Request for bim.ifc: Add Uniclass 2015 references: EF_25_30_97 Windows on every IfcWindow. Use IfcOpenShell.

First a look at what the model holds.

```python
import ifcopenshell

model = ifcopenshell.open("bim.ifc")
print(model.schema)
print("classifications:", [c.Name for c in model.by_type("IfcClassification")])
for ifc_class in ("IfcDoor", "IfcRoof", "IfcStair", "IfcWall", "IfcWindow"):
    print(ifc_class, len(model.by_type(ifc_class)))
```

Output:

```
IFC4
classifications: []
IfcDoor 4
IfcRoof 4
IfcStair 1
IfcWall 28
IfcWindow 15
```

```python
import ifcopenshell
import ifcopenshell.api.classification

model = ifcopenshell.open("bim.ifc")

system = ifcopenshell.api.classification.add_classification(model, classification="Uniclass 2015")

codes = {
    "IfcWindow": ("EF_25_30_97", "Windows"),
}
for ifc_class, (code, name) in codes.items():
    products = model.by_type(ifc_class)
    ifcopenshell.api.classification.add_reference(
        model, products=products, classification=system, identification=code, name=name
    )
    print(code, len(products))

model.write("bim_edited.ifc")
```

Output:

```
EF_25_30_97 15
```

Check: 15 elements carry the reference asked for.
